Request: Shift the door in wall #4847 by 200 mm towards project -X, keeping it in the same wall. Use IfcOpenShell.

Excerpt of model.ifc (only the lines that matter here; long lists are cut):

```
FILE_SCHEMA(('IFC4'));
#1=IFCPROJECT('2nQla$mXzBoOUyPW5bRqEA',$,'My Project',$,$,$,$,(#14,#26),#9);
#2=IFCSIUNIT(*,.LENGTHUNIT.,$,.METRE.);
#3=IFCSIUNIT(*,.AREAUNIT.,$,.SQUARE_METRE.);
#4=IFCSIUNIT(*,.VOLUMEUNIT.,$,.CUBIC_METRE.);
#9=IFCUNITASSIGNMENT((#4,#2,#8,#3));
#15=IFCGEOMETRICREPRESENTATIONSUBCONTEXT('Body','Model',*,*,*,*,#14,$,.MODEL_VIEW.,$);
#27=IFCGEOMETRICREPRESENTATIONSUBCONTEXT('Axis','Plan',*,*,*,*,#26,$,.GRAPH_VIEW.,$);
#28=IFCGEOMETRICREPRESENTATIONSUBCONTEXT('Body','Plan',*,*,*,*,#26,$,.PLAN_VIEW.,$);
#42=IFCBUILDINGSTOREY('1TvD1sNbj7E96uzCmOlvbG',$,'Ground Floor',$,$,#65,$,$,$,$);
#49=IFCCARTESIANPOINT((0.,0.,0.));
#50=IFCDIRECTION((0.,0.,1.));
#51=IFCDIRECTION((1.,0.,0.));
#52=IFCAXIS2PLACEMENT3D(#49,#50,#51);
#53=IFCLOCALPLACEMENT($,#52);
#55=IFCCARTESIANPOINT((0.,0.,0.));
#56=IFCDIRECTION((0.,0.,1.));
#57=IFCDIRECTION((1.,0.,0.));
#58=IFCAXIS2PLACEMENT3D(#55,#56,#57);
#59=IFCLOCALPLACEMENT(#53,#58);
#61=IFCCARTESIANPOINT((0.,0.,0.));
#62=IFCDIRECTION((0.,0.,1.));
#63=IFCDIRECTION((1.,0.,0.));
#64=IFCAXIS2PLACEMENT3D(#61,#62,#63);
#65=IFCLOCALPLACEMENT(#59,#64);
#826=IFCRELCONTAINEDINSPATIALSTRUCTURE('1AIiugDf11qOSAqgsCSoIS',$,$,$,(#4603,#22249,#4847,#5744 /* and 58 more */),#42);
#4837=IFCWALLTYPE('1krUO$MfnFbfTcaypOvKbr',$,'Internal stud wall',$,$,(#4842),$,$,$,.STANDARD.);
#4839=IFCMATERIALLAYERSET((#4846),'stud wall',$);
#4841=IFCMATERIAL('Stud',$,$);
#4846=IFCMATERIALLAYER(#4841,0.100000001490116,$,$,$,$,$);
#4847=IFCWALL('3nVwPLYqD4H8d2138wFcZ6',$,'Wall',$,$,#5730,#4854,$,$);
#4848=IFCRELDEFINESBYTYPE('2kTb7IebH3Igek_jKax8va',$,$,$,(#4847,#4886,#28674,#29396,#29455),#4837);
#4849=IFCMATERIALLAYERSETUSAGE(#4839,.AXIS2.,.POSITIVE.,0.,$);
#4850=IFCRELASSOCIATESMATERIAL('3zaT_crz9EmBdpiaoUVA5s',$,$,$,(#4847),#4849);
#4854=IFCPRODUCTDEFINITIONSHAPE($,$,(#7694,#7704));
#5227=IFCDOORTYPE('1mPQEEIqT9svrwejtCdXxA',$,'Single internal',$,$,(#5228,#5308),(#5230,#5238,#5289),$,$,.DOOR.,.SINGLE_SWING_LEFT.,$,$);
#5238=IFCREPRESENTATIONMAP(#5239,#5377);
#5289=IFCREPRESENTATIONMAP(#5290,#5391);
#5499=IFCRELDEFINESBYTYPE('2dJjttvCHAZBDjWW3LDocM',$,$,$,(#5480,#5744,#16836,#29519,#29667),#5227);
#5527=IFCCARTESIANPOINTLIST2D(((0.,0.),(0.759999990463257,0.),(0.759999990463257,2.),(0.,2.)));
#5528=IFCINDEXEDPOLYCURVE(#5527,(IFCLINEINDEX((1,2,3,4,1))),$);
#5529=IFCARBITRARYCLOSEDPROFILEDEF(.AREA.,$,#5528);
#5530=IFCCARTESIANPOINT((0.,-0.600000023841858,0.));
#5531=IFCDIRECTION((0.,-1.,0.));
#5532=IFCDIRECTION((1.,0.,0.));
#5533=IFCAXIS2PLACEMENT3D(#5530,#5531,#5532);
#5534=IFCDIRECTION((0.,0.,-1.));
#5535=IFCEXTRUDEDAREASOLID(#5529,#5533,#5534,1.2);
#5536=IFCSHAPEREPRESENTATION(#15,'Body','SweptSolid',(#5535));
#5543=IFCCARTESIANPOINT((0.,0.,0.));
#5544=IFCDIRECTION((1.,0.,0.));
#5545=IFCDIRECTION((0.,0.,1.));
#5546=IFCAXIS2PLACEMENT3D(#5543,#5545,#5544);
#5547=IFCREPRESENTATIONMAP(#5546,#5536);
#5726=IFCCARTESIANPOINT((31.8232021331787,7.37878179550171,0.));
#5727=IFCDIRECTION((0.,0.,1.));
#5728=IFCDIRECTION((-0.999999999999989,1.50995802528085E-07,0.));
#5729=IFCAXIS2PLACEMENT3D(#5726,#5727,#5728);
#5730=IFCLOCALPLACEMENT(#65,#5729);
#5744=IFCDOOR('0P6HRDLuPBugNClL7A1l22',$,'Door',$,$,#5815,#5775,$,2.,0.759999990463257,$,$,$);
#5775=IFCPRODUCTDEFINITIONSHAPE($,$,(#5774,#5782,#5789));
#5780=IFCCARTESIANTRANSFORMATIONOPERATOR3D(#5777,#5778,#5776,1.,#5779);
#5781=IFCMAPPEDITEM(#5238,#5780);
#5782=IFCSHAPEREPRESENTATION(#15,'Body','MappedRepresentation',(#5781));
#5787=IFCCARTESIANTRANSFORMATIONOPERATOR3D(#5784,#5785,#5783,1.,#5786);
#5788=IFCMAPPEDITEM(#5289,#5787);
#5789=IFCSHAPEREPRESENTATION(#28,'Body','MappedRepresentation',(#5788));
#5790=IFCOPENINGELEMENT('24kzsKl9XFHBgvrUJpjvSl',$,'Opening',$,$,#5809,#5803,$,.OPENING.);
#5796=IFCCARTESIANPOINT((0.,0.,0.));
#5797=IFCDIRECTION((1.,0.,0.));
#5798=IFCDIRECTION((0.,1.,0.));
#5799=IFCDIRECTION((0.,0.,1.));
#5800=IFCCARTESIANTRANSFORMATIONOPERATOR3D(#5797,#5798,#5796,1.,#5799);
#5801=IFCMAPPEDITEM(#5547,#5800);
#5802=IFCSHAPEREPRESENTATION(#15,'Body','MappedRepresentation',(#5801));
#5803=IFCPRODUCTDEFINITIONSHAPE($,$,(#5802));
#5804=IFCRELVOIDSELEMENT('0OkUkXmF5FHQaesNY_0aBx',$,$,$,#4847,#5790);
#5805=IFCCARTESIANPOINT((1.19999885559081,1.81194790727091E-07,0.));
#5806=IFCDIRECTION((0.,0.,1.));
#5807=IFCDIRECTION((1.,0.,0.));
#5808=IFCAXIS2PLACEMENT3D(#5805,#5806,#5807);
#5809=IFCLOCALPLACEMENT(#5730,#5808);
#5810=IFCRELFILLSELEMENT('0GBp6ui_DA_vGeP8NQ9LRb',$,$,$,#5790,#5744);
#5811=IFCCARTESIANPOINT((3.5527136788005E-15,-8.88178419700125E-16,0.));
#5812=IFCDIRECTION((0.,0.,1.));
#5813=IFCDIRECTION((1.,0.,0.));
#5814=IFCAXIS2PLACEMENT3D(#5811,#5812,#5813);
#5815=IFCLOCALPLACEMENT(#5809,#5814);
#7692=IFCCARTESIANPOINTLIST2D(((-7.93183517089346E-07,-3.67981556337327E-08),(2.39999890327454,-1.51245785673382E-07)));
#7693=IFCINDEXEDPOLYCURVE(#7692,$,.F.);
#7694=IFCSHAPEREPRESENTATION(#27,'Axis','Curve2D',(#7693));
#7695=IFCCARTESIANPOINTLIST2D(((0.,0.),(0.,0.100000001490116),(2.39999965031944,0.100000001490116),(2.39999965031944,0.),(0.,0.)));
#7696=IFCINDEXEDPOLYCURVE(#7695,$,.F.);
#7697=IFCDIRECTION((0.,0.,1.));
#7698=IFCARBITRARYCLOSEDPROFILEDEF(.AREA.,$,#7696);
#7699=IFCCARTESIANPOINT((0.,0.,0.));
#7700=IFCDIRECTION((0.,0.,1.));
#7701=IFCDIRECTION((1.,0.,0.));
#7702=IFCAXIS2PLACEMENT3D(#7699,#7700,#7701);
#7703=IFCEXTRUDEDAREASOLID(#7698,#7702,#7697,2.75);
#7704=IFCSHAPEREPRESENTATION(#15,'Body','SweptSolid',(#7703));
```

```python
import ifcopenshell
import ifcopenshell.api.geometry
import ifcopenshell.util.placement

model = ifcopenshell.open("model.ifc")

door = model.by_guid("0P6HRDLuPBugNClL7A1l22")
opening = door.FillsVoids[0].RelatingOpeningElement
wall = opening.VoidsElements[0].RelatingBuildingElement

wall_matrix = ifcopenshell.util.placement.get_local_placement(wall.ObjectPlacement)
shift = wall_matrix[:3, 0] * 0.2
before = ifcopenshell.util.placement.get_local_placement(door.ObjectPlacement)[:3, 3].copy()

# The door is placed relative to its opening, so it follows when the opening moves.
matrix = ifcopenshell.util.placement.get_local_placement(opening.ObjectPlacement)
matrix[:3, 3] += shift
ifcopenshell.api.geometry.edit_object_placement(
    model, product=opening, matrix=matrix, is_si=False, should_transform_children=True
)

after = ifcopenshell.util.placement.get_local_placement(door.ObjectPlacement)[:3, 3]
print("door moved by", (after - before).round(3) + 0.0)

model.write("model_edited.ifc")
```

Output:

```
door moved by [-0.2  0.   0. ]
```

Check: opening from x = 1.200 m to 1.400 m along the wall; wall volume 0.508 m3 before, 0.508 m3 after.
